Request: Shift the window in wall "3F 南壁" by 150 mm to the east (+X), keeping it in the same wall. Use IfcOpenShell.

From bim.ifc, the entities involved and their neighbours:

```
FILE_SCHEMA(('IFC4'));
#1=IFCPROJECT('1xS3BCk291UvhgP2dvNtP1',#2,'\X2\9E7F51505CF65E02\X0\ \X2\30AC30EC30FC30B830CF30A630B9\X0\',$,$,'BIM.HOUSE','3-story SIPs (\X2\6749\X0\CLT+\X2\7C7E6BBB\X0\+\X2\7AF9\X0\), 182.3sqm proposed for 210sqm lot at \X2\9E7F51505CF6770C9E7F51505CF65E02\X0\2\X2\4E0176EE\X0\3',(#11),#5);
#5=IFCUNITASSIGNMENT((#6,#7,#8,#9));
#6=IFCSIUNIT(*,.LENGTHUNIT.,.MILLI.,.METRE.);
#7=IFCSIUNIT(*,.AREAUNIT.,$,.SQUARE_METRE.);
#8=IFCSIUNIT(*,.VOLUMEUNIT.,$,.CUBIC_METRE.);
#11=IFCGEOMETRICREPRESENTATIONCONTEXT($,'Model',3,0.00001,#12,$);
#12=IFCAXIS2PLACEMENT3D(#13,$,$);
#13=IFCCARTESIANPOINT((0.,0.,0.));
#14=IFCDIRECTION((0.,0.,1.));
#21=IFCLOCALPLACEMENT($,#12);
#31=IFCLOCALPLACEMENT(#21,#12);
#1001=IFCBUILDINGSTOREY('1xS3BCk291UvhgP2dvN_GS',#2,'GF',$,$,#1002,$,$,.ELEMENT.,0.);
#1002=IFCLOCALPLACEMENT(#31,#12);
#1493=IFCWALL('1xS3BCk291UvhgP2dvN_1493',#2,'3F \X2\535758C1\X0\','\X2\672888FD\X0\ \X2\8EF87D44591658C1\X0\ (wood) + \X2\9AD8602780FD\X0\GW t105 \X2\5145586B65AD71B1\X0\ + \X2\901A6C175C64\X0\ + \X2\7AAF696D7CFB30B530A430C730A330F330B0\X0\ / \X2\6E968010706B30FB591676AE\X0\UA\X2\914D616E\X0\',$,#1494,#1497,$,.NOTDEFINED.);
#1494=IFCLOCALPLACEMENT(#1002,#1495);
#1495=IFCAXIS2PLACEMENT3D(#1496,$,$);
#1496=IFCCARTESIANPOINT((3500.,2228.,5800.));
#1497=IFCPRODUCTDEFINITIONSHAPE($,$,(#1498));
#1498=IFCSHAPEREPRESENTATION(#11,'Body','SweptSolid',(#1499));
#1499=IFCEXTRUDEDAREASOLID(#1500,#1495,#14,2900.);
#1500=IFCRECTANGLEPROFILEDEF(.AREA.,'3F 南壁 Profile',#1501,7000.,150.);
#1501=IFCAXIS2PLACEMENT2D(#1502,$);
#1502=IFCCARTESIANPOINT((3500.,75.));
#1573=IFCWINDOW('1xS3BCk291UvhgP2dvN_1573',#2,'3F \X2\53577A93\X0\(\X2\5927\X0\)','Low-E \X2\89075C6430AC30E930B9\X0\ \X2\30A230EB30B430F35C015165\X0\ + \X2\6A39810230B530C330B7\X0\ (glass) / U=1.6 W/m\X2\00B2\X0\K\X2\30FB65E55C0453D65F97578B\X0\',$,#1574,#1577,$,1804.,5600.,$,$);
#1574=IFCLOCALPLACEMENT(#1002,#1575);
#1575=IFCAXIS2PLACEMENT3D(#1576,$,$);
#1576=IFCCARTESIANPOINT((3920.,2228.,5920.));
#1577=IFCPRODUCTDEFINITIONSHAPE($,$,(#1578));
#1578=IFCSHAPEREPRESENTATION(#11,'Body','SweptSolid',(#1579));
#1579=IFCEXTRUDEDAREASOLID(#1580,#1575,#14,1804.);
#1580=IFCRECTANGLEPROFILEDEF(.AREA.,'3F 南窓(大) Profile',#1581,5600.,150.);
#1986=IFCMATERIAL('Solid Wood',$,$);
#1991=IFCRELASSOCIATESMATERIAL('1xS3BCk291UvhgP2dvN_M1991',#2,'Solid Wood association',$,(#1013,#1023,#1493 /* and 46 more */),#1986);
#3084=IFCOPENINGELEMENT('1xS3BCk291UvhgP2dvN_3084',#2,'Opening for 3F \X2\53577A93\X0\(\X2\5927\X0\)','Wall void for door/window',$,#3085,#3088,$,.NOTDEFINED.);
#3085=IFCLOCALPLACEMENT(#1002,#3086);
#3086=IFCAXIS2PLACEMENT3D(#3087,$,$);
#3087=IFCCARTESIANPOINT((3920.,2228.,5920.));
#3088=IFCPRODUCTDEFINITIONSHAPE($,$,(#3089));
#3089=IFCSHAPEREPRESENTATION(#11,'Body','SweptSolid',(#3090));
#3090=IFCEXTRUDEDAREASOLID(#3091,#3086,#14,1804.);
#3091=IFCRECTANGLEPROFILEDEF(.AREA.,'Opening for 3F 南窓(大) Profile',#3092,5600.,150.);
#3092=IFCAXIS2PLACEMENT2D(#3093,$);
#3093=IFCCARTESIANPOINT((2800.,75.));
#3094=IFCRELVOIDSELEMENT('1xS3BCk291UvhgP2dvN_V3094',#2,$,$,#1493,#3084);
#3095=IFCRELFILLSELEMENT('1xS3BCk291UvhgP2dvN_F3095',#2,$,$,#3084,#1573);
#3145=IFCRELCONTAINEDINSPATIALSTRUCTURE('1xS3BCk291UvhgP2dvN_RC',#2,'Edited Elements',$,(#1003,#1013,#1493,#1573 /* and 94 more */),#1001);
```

```python
import ifcopenshell
import ifcopenshell.api.geometry
import ifcopenshell.util.placement

model = ifcopenshell.open("bim.ifc")

window = model.by_id(1573)
opening = window.FillsVoids[0].RelatingOpeningElement
wall = opening.VoidsElements[0].RelatingBuildingElement

wall_matrix = ifcopenshell.util.placement.get_local_placement(wall.ObjectPlacement)
shift = wall_matrix[:3, 0] * 150.0
before = ifcopenshell.util.placement.get_local_placement(window.ObjectPlacement)[:3, 3].copy()

# The window is not placed relative to its opening, so move both.
for product in (opening, window):
    matrix = ifcopenshell.util.placement.get_local_placement(product.ObjectPlacement)
    matrix[:3, 3] += shift
    ifcopenshell.api.geometry.edit_object_placement(model, product=product, matrix=matrix, is_si=False)

after = ifcopenshell.util.placement.get_local_placement(window.ObjectPlacement)[:3, 3]
print("window moved by", (after - before).round(3) + 0.0)

model.write("bim_v2.ifc")
```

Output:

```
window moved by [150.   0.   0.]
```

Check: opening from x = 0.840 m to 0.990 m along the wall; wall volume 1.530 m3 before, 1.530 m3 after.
